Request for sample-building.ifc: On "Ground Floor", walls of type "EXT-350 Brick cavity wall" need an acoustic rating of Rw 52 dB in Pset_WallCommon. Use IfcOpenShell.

First a look at what the model holds.

```python
import ifcopenshell
import ifcopenshell.util.element

model = ifcopenshell.open("sample-building.ifc")
print(model.schema)
storey = next(s for s in model.by_type("IfcBuildingStorey") if s.Name == "Ground Floor")
walls = [e for e in ifcopenshell.util.element.get_decomposition(storey) if e.is_a("IfcWall")]
seen = {}
for e in walls:
    element_type = ifcopenshell.util.element.get_type(e)
    key = (element_type.Name if element_type != e and element_type else None, ifcopenshell.util.element.get_pset(e, "Pset_WallCommon", "AcousticRating"))
    seen[key] = seen.get(key, 0) + 1
for (name, value), count in sorted(seen.items(), key=str):
    print(count, "x", name, "|", value)
```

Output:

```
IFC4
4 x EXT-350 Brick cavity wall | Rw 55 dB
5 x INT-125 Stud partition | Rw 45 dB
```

```python
import ifcopenshell
import ifcopenshell.api.pset
import ifcopenshell.util.element

model = ifcopenshell.open("sample-building.ifc")

storey = next(s for s in model.by_type("IfcBuildingStorey") if s.Name == "Ground Floor")
walls = [e for e in ifcopenshell.util.element.get_decomposition(storey) if e.is_a("IfcWall")]

count = 0
for e in walls:
    element_type = ifcopenshell.util.element.get_type(e)
    if element_type in (None, e) or element_type.Name != "EXT-350 Brick cavity wall":
        continue
    # add_pset returns the element's existing set when there is one.
    pset = ifcopenshell.api.pset.add_pset(model, product=e, name="Pset_WallCommon")
    ifcopenshell.api.pset.edit_pset(model, pset=pset, properties={"AcousticRating": "Rw 52 dB"})
    count += 1

print(count, "walls updated")

model.write("sample-building_v2.ifc")
```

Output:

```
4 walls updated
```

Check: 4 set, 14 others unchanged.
